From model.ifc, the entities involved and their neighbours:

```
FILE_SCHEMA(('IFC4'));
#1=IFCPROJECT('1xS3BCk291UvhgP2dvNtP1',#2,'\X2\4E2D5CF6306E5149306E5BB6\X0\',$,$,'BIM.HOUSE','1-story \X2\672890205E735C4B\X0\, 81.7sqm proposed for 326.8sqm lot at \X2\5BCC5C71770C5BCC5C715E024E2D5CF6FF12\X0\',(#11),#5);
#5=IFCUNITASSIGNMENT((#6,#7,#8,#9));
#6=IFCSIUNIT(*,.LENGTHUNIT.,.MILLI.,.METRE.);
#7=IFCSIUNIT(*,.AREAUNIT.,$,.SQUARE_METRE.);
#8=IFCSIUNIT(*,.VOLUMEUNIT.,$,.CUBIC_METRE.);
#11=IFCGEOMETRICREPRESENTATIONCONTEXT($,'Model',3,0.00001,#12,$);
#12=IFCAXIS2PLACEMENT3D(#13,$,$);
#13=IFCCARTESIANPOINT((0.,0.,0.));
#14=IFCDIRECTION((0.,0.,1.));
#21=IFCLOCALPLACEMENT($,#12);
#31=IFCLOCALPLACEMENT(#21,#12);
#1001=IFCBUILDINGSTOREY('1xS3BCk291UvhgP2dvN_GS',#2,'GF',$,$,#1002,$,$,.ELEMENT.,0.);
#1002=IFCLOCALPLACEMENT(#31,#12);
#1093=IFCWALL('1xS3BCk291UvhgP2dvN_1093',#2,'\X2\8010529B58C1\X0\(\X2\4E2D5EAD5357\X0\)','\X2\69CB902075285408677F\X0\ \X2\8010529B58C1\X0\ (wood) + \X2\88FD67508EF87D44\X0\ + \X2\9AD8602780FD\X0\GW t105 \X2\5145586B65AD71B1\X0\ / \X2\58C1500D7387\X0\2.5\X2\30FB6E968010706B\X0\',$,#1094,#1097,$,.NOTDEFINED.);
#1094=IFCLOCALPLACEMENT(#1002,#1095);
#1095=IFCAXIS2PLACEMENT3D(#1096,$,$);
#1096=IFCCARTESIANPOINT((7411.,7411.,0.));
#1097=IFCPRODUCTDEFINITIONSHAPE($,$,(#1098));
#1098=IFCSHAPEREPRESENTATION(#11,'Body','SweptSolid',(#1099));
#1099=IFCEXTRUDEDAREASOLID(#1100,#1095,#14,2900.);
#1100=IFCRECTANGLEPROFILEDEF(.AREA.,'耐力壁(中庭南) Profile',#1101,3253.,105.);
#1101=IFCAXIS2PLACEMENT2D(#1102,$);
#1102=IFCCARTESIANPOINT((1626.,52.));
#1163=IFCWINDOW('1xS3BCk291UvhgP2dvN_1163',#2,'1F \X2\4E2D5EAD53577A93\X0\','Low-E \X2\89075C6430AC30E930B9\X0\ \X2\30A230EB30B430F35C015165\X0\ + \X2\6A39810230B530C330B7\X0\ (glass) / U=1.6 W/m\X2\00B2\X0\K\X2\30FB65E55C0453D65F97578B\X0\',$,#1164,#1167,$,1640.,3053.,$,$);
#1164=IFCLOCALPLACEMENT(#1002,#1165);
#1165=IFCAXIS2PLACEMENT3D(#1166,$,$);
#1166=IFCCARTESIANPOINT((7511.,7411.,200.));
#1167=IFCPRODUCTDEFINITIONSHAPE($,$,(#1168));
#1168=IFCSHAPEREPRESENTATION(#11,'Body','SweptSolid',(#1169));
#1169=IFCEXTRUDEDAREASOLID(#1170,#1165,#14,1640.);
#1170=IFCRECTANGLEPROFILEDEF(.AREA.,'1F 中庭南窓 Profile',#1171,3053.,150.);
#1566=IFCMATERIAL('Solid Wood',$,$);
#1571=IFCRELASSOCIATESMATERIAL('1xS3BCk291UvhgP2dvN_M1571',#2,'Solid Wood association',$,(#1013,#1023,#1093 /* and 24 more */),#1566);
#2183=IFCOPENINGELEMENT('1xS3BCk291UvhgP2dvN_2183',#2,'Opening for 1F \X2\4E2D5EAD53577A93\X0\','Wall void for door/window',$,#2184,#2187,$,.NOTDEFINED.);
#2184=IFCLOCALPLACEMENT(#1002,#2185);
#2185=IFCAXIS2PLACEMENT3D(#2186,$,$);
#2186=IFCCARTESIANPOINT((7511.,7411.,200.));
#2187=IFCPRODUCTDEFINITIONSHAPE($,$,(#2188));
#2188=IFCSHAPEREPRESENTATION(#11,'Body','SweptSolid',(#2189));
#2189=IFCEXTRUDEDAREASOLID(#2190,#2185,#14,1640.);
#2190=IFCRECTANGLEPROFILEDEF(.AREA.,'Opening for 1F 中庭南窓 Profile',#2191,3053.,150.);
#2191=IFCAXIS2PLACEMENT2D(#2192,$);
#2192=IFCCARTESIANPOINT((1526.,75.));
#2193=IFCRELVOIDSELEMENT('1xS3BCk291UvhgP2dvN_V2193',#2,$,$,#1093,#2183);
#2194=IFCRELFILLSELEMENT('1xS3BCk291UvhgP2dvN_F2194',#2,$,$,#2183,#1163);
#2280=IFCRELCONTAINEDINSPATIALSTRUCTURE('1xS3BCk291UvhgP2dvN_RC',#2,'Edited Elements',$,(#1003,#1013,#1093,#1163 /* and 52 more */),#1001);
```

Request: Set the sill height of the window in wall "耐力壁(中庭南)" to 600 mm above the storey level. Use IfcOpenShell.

```python
import numpy as np
import ifcopenshell
import ifcopenshell.api.geometry
import ifcopenshell.geom
import ifcopenshell.util.element
import ifcopenshell.util.placement
import ifcopenshell.util.shape
import ifcopenshell.util.unit

model = ifcopenshell.open("model.ifc")
unit_scale = ifcopenshell.util.unit.calculate_unit_scale(model)

window = model.by_id(1163)
opening = window.FillsVoids[0].RelatingOpeningElement
storey = ifcopenshell.util.element.get_container(window, ifc_class="IfcBuildingStorey")
level = ifcopenshell.util.placement.get_local_placement(storey.ObjectPlacement)[2, 3]

# The opening's origin need not be at the sill, so measure its lowest point.
shape = ifcopenshell.geom.create_shape(ifcopenshell.geom.settings(), opening)
bottom = ifcopenshell.util.shape.get_shape_bottom_elevation(shape, shape.geometry) / unit_scale
dz = level + 0.6 / unit_scale - bottom

shift = np.array([0.0, 0.0, dz])
# The window is not placed relative to its opening, so move both.
for product in (opening, window):
    matrix = ifcopenshell.util.placement.get_local_placement(product.ObjectPlacement)
    matrix[:3, 3] += shift
    ifcopenshell.api.geometry.edit_object_placement(model, product=product, matrix=matrix, is_si=False)

print(f"moved by {dz * unit_scale:+.3f} m")

model.write("model-out.ifc")
```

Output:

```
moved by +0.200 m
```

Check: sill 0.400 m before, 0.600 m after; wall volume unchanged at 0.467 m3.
